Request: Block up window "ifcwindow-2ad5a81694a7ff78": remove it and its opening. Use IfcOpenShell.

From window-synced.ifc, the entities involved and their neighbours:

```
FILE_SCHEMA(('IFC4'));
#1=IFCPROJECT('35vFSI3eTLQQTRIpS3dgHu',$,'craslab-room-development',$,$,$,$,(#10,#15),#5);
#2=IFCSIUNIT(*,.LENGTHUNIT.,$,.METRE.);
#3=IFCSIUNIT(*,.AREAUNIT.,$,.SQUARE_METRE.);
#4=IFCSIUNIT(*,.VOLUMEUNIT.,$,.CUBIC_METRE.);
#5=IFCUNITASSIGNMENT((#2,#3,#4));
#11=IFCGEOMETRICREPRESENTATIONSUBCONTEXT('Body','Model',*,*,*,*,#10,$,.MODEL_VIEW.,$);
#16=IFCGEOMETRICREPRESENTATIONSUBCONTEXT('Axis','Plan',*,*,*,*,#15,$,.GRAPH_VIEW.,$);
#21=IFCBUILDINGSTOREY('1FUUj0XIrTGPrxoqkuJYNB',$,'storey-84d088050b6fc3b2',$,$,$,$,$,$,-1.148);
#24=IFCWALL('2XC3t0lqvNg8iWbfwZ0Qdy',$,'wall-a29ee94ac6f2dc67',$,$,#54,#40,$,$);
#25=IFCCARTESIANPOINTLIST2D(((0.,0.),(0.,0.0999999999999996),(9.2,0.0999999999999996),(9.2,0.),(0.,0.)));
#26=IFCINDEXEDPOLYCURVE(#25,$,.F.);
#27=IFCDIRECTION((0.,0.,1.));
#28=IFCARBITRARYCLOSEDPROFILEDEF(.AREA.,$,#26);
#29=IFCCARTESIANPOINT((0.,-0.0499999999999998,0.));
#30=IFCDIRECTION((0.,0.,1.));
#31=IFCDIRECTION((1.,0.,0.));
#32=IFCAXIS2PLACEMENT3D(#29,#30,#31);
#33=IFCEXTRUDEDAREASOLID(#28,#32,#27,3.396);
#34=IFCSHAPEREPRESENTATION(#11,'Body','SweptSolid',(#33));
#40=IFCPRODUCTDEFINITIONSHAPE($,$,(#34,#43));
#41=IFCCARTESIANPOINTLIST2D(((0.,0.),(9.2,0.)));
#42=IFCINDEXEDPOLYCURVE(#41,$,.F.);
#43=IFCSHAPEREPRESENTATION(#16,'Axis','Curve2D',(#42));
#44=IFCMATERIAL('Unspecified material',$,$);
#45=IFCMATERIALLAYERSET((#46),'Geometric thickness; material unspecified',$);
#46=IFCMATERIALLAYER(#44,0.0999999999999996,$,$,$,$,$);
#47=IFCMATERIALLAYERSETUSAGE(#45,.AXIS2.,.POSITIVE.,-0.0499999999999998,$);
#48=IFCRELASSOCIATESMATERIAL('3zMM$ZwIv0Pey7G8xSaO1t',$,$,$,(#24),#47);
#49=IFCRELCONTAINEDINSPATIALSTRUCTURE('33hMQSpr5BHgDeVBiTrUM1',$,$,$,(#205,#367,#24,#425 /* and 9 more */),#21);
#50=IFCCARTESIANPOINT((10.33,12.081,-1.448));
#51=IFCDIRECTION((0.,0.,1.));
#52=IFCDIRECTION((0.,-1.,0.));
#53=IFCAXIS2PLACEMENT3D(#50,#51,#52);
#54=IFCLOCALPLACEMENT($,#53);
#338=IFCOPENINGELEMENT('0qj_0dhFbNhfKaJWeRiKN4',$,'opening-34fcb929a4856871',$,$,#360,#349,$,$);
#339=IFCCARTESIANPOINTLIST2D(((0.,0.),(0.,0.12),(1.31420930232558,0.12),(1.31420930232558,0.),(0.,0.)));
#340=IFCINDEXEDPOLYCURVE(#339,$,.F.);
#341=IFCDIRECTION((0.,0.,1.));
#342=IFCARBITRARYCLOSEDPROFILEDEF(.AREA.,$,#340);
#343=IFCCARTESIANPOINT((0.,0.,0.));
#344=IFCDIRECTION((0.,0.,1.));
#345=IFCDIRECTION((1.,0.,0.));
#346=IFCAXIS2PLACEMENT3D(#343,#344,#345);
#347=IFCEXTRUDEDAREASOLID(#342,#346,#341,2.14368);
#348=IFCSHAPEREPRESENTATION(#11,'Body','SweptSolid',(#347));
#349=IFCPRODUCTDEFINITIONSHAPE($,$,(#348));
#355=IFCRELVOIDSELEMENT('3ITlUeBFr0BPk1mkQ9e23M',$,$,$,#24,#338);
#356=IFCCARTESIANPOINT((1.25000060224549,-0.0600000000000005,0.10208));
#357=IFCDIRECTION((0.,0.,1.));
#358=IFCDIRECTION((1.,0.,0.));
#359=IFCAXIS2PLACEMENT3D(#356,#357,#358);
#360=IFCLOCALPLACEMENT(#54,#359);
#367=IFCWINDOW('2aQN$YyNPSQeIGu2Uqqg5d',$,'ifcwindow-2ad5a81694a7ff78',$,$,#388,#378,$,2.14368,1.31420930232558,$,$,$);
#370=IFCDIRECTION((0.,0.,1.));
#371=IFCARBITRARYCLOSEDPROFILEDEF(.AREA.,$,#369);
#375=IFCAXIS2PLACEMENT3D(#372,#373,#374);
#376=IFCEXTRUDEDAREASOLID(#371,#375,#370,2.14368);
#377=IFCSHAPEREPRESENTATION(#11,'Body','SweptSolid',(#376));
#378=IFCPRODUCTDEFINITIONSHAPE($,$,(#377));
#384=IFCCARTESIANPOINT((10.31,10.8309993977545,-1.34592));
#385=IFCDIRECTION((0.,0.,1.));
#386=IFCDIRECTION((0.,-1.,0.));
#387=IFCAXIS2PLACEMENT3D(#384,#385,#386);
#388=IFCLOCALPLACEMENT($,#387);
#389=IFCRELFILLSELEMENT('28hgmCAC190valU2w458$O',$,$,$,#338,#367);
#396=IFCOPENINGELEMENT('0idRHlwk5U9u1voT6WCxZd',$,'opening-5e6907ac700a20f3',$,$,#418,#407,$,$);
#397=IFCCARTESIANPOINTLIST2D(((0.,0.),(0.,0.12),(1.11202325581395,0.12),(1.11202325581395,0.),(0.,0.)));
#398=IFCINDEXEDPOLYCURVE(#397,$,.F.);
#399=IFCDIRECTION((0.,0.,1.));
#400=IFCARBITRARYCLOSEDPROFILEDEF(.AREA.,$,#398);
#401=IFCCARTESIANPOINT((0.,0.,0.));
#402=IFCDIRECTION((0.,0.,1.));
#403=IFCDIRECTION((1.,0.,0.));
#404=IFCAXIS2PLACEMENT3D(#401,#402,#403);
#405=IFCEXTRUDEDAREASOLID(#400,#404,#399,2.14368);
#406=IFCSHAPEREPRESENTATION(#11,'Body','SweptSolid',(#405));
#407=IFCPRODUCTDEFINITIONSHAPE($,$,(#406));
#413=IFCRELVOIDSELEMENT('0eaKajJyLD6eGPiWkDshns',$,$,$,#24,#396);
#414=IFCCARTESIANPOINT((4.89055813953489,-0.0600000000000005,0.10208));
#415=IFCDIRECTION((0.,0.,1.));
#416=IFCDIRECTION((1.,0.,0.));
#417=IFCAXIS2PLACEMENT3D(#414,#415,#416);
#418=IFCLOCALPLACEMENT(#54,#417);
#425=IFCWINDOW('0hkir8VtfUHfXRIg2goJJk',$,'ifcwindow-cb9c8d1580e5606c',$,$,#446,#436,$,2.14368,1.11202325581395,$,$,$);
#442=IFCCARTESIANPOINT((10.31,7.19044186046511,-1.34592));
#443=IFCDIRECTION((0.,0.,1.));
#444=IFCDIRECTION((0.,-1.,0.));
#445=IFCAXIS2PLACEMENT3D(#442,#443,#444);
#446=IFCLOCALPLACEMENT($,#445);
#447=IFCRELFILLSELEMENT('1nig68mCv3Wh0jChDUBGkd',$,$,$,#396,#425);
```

```python
import ifcopenshell
import ifcopenshell.api.feature
import ifcopenshell.api.root
import ifcopenshell.geom
import ifcopenshell.util.shape

model = ifcopenshell.open("window-synced.ifc")
settings = ifcopenshell.geom.settings()


def volume(element):
    """Net volume in cubic metres, openings subtracted."""
    shape = ifcopenshell.geom.create_shape(settings, element)
    return ifcopenshell.util.shape.get_volume(shape.geometry)


window = model.by_guid("2aQN$YyNPSQeIGu2Uqqg5d")
opening = window.FillsVoids[0].RelatingOpeningElement
wall = opening.VoidsElements[0].RelatingBuildingElement
before = volume(wall)

ifcopenshell.api.root.remove_product(model, product=window)
ifcopenshell.api.feature.remove_feature(model, feature=opening)

after = volume(wall)

print(f"wall volume {before:.3f} -> {after:.3f} m3")

model.write("window-synced-out.ifc")
```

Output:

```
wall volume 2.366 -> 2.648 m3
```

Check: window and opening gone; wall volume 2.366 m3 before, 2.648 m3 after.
